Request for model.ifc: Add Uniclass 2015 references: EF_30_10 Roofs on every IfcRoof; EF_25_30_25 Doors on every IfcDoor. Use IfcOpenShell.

First a look at what the model holds.

```python
import ifcopenshell

model = ifcopenshell.open("model.ifc")
print(model.schema)
print("classifications:", [c.Name for c in model.by_type("IfcClassification")])
for ifc_class in ("IfcDoor", "IfcRoof", "IfcStair", "IfcWall", "IfcWindow"):
    print(ifc_class, len(model.by_type(ifc_class)))
```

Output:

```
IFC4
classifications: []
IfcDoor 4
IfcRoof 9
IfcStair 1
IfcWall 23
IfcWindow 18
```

```python
import ifcopenshell
import ifcopenshell.api.classification

model = ifcopenshell.open("model.ifc")

system = ifcopenshell.api.classification.add_classification(model, classification="Uniclass 2015")

codes = {
    "IfcRoof": ("EF_30_10", "Roofs"),
    "IfcDoor": ("EF_25_30_25", "Doors"),
}
for ifc_class, (code, name) in codes.items():
    products = model.by_type(ifc_class)
    ifcopenshell.api.classification.add_reference(
        model, products=products, classification=system, identification=code, name=name
    )
    print(code, len(products))

model.write("model_v2.ifc")
```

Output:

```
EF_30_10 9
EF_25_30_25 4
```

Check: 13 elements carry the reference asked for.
